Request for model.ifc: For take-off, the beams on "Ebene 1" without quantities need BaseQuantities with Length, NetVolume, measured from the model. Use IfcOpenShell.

First a look at what the model holds.

```python
import ifcopenshell
import ifcopenshell.util.element
import ifcopenshell.util.unit

model = ifcopenshell.open("model.ifc")
print(model.schema)
for unit_type in ("LENGTHUNIT", "AREAUNIT", "VOLUMEUNIT"):
    print(unit_type, ifcopenshell.util.unit.calculate_unit_scale(model, unit_type))
storey = next(s for s in model.by_type("IfcBuildingStorey") if s.Name == "Ebene 1")
beams = [e for e in ifcopenshell.util.element.get_decomposition(storey) if e.is_a("IfcBeam")]
for e in sorted(beams, key=lambda e: e.id()):
    print(e.id(), e.is_a(), e.Name, list(ifcopenshell.util.element.get_psets(e, qtos_only=True)), sep=" | ")
```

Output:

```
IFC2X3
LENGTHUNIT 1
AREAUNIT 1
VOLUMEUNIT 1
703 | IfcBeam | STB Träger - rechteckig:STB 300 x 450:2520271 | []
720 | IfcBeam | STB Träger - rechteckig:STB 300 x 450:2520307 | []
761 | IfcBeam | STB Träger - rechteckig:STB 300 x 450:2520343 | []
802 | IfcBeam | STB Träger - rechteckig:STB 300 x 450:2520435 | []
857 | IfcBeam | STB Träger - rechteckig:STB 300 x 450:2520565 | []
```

```python
import ifcopenshell
import ifcopenshell.api.pset
import ifcopenshell.geom
import ifcopenshell.util.element
import ifcopenshell.util.shape
import ifcopenshell.util.unit

model = ifcopenshell.open("model.ifc")
unit_scale = ifcopenshell.util.unit.calculate_unit_scale(model)
volume_scale = ifcopenshell.util.unit.calculate_unit_scale(model, "VOLUMEUNIT")
settings = ifcopenshell.geom.settings()

storey = next(s for s in model.by_type("IfcBuildingStorey") if s.Name == "Ebene 1")
beams = [e for e in ifcopenshell.util.element.get_decomposition(storey) if e.is_a("IfcBeam")]

for e in sorted(beams, key=lambda e: e.id()):
    if ifcopenshell.util.element.get_psets(e, qtos_only=True, should_inherit=False):
        continue
    # Geometry comes back in metres, in the element's own axes.
    shape = ifcopenshell.geom.create_shape(settings, e)
    values = {
        "Length": ifcopenshell.util.shape.get_max_xyz(shape.geometry) / unit_scale,
        "NetVolume": ifcopenshell.util.shape.get_volume(shape.geometry) / volume_scale,
    }
    qto = ifcopenshell.api.pset.add_qto(model, product=e, name="BaseQuantities")
    ifcopenshell.api.pset.edit_qto(model, qto=qto, properties=values)
    print(e.id(), {k: round(v, 3) for k, v in values.items()})

model.write("model_v2.ifc")
```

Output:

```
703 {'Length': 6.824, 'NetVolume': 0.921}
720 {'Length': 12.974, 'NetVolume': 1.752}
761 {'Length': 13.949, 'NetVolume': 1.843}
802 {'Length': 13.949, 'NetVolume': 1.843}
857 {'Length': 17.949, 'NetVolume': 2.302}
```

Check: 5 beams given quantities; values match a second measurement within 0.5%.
